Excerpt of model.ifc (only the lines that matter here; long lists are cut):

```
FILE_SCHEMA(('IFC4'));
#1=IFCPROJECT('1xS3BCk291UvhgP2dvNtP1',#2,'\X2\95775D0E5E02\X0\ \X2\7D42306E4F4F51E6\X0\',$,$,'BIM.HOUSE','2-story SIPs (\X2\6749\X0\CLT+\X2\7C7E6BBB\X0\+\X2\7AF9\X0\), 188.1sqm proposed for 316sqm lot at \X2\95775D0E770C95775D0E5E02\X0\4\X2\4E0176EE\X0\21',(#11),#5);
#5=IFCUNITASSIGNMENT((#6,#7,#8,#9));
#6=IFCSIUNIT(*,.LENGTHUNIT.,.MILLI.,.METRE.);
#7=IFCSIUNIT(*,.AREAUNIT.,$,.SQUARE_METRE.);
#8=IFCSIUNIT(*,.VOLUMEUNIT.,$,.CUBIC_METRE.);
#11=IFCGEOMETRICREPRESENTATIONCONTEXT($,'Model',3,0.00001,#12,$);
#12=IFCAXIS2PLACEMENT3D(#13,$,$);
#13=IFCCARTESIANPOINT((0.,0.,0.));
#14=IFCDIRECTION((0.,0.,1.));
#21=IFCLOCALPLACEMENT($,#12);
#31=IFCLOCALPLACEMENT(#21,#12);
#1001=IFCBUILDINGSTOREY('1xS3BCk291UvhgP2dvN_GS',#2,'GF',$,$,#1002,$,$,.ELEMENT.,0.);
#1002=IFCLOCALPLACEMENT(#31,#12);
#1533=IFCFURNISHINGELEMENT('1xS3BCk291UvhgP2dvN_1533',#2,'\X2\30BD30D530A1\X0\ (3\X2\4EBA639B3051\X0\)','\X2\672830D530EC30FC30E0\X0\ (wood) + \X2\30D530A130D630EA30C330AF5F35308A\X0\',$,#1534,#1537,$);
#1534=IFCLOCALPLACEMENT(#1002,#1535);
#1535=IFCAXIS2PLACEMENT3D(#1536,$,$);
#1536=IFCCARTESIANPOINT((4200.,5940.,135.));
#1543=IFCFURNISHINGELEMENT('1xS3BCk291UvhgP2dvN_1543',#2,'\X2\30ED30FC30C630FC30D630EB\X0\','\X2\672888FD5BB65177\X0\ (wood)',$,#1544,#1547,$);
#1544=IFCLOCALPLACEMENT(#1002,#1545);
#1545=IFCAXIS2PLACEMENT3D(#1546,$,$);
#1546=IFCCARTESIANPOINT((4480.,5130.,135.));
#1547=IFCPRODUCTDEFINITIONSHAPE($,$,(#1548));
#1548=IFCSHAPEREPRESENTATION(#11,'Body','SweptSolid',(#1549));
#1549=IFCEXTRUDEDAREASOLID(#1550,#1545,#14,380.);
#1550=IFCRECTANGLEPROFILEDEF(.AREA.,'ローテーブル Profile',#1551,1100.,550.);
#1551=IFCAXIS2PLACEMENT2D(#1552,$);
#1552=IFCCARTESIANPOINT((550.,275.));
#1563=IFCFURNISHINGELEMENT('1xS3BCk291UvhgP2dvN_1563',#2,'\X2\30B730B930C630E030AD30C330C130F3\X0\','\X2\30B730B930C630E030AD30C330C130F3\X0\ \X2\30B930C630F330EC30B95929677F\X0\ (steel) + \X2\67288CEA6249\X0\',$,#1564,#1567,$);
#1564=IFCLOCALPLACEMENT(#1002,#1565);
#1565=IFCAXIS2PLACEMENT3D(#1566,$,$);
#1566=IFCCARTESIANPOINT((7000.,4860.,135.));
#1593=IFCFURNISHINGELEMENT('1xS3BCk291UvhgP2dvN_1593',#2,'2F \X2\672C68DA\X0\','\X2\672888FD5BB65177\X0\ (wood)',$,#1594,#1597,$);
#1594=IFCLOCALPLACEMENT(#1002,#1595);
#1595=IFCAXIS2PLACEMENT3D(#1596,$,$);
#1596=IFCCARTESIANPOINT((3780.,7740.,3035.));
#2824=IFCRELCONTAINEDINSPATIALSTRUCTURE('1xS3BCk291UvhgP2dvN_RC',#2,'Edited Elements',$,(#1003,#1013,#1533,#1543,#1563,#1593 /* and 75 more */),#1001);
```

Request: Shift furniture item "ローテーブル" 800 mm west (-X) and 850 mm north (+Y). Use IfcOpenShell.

```python
import ifcopenshell
import ifcopenshell.api.geometry
import ifcopenshell.util.placement

model = ifcopenshell.open("model.ifc")

item = model.by_guid("1xS3BCk291UvhgP2dvN_1543")
matrix = ifcopenshell.util.placement.get_local_placement(item.ObjectPlacement)
matrix[0, 3] -= 800.0
matrix[1, 3] += 850.0
ifcopenshell.api.geometry.edit_object_placement(model, product=item, matrix=matrix, is_si=False)

print(ifcopenshell.util.placement.get_local_placement(item.ObjectPlacement).round(3) + 0.0)

model.write("model_updated.ifc")
```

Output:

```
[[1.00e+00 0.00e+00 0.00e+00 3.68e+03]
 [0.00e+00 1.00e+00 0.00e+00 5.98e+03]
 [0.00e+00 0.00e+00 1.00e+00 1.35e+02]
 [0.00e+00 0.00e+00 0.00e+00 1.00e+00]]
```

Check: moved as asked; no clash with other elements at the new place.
